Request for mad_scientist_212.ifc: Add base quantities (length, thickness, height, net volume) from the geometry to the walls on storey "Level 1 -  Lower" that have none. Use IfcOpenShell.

First a look at what the model holds.

```python
import ifcopenshell
import ifcopenshell.util.element
import ifcopenshell.util.unit

model = ifcopenshell.open("mad_scientist_212.ifc")
print(model.schema)
for unit_type in ("LENGTHUNIT", "AREAUNIT", "VOLUMEUNIT"):
    print(unit_type, ifcopenshell.util.unit.calculate_unit_scale(model, unit_type))
storey = next(s for s in model.by_type("IfcBuildingStorey") if s.Name == "Level 1 -  Lower")
walls = [e for e in ifcopenshell.util.element.get_decomposition(storey) if e.is_a("IfcWall")]
for e in sorted(walls, key=lambda e: e.id()):
    print(e.id(), e.is_a(), e.Name, list(ifcopenshell.util.element.get_psets(e, qtos_only=True)), sep=" | ")
```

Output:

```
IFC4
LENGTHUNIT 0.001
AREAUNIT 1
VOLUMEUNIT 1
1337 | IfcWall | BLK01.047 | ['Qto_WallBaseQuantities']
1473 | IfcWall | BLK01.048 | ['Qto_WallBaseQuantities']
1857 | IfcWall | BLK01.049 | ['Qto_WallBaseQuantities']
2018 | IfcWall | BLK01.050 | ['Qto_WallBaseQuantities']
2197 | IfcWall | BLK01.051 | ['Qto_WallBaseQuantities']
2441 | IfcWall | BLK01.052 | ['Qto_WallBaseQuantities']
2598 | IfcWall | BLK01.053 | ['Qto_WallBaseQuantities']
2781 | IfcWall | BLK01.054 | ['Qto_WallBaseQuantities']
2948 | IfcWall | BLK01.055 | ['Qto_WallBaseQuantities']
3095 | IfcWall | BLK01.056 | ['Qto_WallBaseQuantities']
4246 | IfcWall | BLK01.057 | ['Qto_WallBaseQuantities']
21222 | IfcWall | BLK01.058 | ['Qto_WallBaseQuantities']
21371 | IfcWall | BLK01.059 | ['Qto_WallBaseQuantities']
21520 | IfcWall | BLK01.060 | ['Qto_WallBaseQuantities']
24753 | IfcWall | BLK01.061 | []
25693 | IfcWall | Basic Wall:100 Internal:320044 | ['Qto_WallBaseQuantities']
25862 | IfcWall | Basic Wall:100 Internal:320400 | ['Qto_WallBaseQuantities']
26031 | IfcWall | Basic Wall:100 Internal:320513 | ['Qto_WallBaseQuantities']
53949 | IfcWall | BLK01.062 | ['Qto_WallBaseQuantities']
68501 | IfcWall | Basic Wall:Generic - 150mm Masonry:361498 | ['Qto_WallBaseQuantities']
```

```python
import ifcopenshell
import ifcopenshell.api.pset
import ifcopenshell.geom
import ifcopenshell.util.element
import ifcopenshell.util.shape
import ifcopenshell.util.unit

model = ifcopenshell.open("mad_scientist_212.ifc")
unit_scale = ifcopenshell.util.unit.calculate_unit_scale(model)
volume_scale = ifcopenshell.util.unit.calculate_unit_scale(model, "VOLUMEUNIT")
settings = ifcopenshell.geom.settings()

storey = next(s for s in model.by_type("IfcBuildingStorey") if s.Name == "Level 1 -  Lower")
walls = [e for e in ifcopenshell.util.element.get_decomposition(storey) if e.is_a("IfcWall")]

for e in sorted(walls, key=lambda e: e.id()):
    if ifcopenshell.util.element.get_psets(e, qtos_only=True, should_inherit=False):
        continue
    # Geometry comes back in metres, in the element's own axes.
    shape = ifcopenshell.geom.create_shape(settings, e)
    values = {
        "Length": ifcopenshell.util.shape.get_x(shape.geometry) / unit_scale,
        "Width": ifcopenshell.util.shape.get_y(shape.geometry) / unit_scale,
        "Height": ifcopenshell.util.shape.get_z(shape.geometry) / unit_scale,
        "NetVolume": ifcopenshell.util.shape.get_volume(shape.geometry) / volume_scale,
    }
    qto = ifcopenshell.api.pset.add_qto(model, product=e, name="Qto_WallBaseQuantities")
    ifcopenshell.api.pset.edit_qto(model, qto=qto, properties=values)
    print(e.id(), {k: round(v, 3) for k, v in values.items()})

model.write("mad_scientist_212_updated.ifc")
```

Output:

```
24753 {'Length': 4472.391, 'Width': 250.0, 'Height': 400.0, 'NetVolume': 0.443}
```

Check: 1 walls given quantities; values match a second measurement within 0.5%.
